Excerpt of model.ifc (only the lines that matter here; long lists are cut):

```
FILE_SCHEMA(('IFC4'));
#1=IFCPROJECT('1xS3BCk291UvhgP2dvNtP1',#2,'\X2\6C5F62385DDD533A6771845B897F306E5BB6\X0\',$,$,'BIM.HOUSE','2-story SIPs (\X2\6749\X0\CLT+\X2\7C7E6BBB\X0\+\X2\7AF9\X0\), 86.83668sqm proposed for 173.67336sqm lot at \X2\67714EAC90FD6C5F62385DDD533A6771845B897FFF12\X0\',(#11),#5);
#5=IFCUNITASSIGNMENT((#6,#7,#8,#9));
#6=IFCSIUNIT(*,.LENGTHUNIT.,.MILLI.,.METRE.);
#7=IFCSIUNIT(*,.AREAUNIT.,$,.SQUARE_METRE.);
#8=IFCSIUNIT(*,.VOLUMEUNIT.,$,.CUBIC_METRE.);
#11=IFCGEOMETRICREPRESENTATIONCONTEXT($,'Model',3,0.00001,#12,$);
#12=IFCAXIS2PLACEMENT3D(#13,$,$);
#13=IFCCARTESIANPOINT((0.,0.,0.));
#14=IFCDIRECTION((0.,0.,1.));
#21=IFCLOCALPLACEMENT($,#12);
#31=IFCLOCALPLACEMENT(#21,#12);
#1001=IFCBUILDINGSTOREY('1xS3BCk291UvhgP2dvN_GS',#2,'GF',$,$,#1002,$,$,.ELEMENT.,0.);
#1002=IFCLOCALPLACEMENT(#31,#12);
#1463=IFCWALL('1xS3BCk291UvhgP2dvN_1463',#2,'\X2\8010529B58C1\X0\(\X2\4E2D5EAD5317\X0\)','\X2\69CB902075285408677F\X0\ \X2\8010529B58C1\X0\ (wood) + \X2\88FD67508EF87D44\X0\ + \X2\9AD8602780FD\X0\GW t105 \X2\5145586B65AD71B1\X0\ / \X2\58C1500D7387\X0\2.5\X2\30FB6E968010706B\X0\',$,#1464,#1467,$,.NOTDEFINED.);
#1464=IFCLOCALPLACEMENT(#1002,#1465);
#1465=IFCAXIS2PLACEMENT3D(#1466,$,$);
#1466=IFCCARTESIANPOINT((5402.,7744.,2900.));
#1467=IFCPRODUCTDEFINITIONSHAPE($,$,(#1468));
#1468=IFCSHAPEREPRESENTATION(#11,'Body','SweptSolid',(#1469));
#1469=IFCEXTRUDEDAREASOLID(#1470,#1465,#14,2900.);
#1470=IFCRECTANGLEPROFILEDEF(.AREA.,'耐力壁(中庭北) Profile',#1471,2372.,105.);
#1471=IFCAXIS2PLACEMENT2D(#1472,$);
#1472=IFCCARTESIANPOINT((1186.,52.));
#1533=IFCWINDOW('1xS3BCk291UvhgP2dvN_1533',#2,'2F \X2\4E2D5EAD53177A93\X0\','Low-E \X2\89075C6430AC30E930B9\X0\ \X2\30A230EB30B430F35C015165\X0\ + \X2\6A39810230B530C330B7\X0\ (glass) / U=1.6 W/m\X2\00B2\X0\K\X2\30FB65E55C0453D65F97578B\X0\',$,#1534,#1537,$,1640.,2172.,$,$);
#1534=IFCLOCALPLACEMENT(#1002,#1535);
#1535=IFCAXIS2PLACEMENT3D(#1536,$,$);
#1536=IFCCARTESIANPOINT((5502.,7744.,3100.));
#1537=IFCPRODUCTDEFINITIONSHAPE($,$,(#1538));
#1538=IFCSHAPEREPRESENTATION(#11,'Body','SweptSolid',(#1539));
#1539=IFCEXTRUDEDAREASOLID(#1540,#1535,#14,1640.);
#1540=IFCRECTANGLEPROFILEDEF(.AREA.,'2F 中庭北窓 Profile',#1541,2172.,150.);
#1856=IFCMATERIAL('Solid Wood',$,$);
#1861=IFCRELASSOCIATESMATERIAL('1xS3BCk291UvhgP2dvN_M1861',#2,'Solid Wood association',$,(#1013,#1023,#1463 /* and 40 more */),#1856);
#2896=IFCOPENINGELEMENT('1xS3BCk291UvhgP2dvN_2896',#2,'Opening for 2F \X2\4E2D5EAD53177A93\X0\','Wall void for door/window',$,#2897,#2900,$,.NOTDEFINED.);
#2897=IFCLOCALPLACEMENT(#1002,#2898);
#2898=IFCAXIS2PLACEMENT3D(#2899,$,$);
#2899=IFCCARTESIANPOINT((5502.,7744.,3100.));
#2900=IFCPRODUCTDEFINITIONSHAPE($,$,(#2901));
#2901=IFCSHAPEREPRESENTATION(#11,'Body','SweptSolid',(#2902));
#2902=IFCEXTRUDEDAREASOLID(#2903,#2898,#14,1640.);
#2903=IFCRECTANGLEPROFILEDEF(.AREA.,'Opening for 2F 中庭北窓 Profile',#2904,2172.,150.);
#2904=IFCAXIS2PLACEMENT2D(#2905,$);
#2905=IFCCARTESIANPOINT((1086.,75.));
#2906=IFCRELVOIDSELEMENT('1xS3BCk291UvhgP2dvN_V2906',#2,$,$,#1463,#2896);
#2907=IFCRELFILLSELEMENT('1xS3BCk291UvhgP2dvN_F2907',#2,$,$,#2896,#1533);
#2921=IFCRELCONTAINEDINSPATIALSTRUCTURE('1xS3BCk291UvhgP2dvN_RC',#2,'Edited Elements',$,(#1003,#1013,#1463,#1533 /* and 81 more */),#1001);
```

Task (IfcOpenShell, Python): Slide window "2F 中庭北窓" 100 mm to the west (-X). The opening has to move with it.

```python
import ifcopenshell
import ifcopenshell.api.geometry
import ifcopenshell.util.placement

model = ifcopenshell.open("model.ifc")

window = model.by_id(1533)
opening = window.FillsVoids[0].RelatingOpeningElement
wall = opening.VoidsElements[0].RelatingBuildingElement

wall_matrix = ifcopenshell.util.placement.get_local_placement(wall.ObjectPlacement)
shift = wall_matrix[:3, 0] * -100.0
before = ifcopenshell.util.placement.get_local_placement(window.ObjectPlacement)[:3, 3].copy()

# The window is not placed relative to its opening, so move both.
for product in (opening, window):
    matrix = ifcopenshell.util.placement.get_local_placement(product.ObjectPlacement)
    matrix[:3, 3] += shift
    ifcopenshell.api.geometry.edit_object_placement(model, product=product, matrix=matrix, is_si=False)

after = ifcopenshell.util.placement.get_local_placement(window.ObjectPlacement)[:3, 3]
print("window moved by", (after - before).round(3) + 0.0)

model.write("model-out.ifc")
```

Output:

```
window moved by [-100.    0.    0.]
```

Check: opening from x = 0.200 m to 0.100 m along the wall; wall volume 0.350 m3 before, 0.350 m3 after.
